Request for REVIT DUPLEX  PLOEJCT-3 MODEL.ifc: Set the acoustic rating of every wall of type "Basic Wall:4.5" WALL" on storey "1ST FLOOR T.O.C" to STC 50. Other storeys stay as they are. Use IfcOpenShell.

First a look at what the model holds.

```python
import ifcopenshell
import ifcopenshell.util.element

model = ifcopenshell.open("REVIT DUPLEX  PLOEJCT-3 MODEL.ifc")
print(model.schema)
storey = next(s for s in model.by_type("IfcBuildingStorey") if s.Name == "1ST FLOOR T.O.C")
walls = [e for e in ifcopenshell.util.element.get_decomposition(storey) if e.is_a("IfcWall")]
seen = {}
for e in walls:
    element_type = ifcopenshell.util.element.get_type(e)
    key = (element_type.Name if element_type != e and element_type else None, ifcopenshell.util.element.get_pset(e, "Pset_WallCommon", "AcousticRating"))
    seen[key] = seen.get(key, 0) + 1
for (name, value), count in sorted(seen.items(), key=str):
    print(count, "x", name, "|", value)
```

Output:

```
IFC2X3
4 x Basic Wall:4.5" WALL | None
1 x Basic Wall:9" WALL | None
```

```python
import ifcopenshell
import ifcopenshell.api.pset
import ifcopenshell.util.element

model = ifcopenshell.open("REVIT DUPLEX  PLOEJCT-3 MODEL.ifc")

storey = next(s for s in model.by_type("IfcBuildingStorey") if s.Name == "1ST FLOOR T.O.C")
walls = [e for e in ifcopenshell.util.element.get_decomposition(storey) if e.is_a("IfcWall")]

count = 0
for e in walls:
    element_type = ifcopenshell.util.element.get_type(e)
    if element_type in (None, e) or element_type.Name != 'Basic Wall:4.5" WALL':
        continue
    # add_pset returns the element's existing set when there is one.
    pset = ifcopenshell.api.pset.add_pset(model, product=e, name="Pset_WallCommon")
    ifcopenshell.api.pset.edit_pset(model, pset=pset, properties={"AcousticRating": "STC 50"})
    count += 1

print(count, "walls updated")

model.write("REVIT DUPLEX  PLOEJCT-3 MODEL_v2.ifc")
```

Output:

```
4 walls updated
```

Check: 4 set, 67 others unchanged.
